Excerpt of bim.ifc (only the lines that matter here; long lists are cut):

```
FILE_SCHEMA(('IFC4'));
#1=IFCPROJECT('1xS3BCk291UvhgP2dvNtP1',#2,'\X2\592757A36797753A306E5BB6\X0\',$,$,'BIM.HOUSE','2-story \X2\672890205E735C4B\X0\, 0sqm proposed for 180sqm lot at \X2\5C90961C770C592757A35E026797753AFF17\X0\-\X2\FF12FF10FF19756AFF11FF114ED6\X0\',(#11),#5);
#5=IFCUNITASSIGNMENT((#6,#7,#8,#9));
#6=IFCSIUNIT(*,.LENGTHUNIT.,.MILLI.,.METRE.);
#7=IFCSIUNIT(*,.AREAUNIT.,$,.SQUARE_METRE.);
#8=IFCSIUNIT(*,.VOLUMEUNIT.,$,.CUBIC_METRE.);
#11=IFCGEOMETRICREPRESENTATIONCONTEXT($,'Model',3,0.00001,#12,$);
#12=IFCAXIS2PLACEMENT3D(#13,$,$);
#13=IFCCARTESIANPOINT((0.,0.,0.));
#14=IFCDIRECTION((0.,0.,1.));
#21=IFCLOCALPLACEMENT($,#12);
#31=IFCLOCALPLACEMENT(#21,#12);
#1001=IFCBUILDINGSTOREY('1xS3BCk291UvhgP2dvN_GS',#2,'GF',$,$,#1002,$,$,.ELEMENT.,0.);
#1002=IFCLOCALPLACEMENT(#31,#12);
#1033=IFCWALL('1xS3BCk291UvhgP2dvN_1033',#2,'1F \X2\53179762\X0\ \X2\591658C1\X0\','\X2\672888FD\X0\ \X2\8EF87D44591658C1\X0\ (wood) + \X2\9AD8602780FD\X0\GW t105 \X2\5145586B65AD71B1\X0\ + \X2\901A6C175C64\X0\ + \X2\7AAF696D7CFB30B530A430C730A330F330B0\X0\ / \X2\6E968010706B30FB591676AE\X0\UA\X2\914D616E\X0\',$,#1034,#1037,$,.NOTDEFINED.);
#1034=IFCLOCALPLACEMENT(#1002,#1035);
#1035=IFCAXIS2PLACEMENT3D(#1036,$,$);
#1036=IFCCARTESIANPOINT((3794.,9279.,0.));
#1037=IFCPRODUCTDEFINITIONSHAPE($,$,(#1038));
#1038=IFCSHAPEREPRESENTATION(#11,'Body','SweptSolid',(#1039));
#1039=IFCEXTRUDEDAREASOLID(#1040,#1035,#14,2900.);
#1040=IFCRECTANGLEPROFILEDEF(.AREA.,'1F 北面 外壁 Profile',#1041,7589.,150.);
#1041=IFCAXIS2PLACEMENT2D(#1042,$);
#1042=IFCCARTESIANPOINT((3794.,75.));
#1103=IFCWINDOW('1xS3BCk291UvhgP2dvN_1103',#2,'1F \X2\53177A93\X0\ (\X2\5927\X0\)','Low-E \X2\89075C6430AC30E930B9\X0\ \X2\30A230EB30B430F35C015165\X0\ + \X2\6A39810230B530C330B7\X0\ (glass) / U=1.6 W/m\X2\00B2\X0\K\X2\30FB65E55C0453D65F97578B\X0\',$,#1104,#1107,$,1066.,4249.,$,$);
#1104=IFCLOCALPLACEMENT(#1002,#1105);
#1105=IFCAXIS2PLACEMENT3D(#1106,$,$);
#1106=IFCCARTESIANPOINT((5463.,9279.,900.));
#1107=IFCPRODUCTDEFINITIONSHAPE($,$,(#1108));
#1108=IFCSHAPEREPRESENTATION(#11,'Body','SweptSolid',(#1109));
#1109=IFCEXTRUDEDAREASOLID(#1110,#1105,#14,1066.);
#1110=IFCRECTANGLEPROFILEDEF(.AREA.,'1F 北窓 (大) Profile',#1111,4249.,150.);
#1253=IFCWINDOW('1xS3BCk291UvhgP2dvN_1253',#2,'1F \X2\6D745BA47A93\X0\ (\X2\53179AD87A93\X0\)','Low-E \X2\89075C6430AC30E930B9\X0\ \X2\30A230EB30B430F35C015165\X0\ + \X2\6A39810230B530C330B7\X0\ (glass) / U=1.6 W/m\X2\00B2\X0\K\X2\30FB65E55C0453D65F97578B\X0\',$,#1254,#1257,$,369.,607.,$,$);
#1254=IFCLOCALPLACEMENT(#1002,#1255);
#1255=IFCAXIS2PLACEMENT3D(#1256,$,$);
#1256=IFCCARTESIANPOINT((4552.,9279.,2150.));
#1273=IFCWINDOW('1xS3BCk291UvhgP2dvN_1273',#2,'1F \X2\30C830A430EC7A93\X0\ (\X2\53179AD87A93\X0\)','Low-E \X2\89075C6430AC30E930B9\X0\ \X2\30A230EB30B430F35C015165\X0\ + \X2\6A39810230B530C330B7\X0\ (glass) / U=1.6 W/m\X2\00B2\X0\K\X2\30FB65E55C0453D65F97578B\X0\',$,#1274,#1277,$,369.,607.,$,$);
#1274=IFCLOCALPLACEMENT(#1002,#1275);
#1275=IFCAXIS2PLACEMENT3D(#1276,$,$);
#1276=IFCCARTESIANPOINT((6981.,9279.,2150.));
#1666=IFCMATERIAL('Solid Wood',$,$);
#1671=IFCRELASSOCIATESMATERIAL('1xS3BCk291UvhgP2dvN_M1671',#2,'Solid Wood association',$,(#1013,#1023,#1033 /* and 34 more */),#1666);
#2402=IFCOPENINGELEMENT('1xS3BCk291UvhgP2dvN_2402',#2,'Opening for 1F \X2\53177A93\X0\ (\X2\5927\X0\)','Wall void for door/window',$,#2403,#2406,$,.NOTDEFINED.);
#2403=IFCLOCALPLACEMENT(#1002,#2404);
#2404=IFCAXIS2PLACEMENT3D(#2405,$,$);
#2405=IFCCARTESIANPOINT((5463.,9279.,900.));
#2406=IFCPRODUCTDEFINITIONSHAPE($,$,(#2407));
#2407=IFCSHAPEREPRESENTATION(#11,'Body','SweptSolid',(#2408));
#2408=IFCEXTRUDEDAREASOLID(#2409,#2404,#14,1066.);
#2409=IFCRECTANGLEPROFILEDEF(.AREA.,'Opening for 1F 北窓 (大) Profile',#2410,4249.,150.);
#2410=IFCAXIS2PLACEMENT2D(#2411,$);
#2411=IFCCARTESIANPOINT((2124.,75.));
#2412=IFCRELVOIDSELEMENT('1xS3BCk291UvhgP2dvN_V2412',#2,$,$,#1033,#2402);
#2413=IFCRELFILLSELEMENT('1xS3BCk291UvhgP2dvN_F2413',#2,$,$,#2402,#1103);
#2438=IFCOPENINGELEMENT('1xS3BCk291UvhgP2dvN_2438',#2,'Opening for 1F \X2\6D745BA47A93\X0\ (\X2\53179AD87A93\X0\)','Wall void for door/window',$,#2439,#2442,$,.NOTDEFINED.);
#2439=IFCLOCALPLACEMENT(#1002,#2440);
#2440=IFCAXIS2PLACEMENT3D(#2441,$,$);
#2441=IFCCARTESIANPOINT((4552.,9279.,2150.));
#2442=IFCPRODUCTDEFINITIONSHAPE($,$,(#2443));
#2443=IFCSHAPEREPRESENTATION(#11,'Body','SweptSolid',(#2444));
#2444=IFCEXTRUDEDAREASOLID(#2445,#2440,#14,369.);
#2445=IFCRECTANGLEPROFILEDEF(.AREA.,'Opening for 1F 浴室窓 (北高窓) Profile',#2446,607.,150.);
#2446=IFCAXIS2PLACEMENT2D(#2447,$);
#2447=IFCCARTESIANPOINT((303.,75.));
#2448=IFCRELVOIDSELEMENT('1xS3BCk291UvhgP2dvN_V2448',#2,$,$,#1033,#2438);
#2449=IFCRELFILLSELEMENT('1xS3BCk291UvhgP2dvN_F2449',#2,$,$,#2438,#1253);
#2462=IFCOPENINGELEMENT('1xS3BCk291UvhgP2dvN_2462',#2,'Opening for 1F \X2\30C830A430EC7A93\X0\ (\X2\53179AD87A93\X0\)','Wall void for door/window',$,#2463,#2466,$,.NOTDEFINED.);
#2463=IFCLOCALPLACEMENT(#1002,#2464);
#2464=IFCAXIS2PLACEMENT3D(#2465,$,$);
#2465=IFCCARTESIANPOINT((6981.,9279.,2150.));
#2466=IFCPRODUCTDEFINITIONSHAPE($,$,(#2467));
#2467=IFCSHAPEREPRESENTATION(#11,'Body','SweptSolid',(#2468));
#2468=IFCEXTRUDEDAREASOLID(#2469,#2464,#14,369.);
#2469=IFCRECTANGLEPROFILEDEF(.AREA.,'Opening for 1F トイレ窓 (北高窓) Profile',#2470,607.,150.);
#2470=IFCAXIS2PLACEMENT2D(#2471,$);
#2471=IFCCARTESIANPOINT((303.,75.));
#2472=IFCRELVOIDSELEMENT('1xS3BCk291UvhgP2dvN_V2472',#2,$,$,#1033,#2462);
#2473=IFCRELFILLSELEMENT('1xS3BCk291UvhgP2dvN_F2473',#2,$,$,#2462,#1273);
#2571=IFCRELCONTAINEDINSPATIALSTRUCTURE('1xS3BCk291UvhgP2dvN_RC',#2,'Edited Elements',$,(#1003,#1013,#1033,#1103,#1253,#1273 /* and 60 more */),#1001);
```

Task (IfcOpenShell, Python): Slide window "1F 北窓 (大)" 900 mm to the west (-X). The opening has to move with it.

```python
import ifcopenshell
import ifcopenshell.api.geometry
import ifcopenshell.util.placement

model = ifcopenshell.open("bim.ifc")

window = model.by_id(1103)
opening = window.FillsVoids[0].RelatingOpeningElement
wall = opening.VoidsElements[0].RelatingBuildingElement

wall_matrix = ifcopenshell.util.placement.get_local_placement(wall.ObjectPlacement)
shift = wall_matrix[:3, 0] * -900.0
before = ifcopenshell.util.placement.get_local_placement(window.ObjectPlacement)[:3, 3].copy()

# The window is not placed relative to its opening, so move both.
for product in (opening, window):
    matrix = ifcopenshell.util.placement.get_local_placement(product.ObjectPlacement)
    matrix[:3, 3] += shift
    ifcopenshell.api.geometry.edit_object_placement(model, product=product, matrix=matrix, is_si=False)

after = ifcopenshell.util.placement.get_local_placement(window.ObjectPlacement)[:3, 3]
print("window moved by", (after - before).round(3) + 0.0)

model.write("bim_updated.ifc")
```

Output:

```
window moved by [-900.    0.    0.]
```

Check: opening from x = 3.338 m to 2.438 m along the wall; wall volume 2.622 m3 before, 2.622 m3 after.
